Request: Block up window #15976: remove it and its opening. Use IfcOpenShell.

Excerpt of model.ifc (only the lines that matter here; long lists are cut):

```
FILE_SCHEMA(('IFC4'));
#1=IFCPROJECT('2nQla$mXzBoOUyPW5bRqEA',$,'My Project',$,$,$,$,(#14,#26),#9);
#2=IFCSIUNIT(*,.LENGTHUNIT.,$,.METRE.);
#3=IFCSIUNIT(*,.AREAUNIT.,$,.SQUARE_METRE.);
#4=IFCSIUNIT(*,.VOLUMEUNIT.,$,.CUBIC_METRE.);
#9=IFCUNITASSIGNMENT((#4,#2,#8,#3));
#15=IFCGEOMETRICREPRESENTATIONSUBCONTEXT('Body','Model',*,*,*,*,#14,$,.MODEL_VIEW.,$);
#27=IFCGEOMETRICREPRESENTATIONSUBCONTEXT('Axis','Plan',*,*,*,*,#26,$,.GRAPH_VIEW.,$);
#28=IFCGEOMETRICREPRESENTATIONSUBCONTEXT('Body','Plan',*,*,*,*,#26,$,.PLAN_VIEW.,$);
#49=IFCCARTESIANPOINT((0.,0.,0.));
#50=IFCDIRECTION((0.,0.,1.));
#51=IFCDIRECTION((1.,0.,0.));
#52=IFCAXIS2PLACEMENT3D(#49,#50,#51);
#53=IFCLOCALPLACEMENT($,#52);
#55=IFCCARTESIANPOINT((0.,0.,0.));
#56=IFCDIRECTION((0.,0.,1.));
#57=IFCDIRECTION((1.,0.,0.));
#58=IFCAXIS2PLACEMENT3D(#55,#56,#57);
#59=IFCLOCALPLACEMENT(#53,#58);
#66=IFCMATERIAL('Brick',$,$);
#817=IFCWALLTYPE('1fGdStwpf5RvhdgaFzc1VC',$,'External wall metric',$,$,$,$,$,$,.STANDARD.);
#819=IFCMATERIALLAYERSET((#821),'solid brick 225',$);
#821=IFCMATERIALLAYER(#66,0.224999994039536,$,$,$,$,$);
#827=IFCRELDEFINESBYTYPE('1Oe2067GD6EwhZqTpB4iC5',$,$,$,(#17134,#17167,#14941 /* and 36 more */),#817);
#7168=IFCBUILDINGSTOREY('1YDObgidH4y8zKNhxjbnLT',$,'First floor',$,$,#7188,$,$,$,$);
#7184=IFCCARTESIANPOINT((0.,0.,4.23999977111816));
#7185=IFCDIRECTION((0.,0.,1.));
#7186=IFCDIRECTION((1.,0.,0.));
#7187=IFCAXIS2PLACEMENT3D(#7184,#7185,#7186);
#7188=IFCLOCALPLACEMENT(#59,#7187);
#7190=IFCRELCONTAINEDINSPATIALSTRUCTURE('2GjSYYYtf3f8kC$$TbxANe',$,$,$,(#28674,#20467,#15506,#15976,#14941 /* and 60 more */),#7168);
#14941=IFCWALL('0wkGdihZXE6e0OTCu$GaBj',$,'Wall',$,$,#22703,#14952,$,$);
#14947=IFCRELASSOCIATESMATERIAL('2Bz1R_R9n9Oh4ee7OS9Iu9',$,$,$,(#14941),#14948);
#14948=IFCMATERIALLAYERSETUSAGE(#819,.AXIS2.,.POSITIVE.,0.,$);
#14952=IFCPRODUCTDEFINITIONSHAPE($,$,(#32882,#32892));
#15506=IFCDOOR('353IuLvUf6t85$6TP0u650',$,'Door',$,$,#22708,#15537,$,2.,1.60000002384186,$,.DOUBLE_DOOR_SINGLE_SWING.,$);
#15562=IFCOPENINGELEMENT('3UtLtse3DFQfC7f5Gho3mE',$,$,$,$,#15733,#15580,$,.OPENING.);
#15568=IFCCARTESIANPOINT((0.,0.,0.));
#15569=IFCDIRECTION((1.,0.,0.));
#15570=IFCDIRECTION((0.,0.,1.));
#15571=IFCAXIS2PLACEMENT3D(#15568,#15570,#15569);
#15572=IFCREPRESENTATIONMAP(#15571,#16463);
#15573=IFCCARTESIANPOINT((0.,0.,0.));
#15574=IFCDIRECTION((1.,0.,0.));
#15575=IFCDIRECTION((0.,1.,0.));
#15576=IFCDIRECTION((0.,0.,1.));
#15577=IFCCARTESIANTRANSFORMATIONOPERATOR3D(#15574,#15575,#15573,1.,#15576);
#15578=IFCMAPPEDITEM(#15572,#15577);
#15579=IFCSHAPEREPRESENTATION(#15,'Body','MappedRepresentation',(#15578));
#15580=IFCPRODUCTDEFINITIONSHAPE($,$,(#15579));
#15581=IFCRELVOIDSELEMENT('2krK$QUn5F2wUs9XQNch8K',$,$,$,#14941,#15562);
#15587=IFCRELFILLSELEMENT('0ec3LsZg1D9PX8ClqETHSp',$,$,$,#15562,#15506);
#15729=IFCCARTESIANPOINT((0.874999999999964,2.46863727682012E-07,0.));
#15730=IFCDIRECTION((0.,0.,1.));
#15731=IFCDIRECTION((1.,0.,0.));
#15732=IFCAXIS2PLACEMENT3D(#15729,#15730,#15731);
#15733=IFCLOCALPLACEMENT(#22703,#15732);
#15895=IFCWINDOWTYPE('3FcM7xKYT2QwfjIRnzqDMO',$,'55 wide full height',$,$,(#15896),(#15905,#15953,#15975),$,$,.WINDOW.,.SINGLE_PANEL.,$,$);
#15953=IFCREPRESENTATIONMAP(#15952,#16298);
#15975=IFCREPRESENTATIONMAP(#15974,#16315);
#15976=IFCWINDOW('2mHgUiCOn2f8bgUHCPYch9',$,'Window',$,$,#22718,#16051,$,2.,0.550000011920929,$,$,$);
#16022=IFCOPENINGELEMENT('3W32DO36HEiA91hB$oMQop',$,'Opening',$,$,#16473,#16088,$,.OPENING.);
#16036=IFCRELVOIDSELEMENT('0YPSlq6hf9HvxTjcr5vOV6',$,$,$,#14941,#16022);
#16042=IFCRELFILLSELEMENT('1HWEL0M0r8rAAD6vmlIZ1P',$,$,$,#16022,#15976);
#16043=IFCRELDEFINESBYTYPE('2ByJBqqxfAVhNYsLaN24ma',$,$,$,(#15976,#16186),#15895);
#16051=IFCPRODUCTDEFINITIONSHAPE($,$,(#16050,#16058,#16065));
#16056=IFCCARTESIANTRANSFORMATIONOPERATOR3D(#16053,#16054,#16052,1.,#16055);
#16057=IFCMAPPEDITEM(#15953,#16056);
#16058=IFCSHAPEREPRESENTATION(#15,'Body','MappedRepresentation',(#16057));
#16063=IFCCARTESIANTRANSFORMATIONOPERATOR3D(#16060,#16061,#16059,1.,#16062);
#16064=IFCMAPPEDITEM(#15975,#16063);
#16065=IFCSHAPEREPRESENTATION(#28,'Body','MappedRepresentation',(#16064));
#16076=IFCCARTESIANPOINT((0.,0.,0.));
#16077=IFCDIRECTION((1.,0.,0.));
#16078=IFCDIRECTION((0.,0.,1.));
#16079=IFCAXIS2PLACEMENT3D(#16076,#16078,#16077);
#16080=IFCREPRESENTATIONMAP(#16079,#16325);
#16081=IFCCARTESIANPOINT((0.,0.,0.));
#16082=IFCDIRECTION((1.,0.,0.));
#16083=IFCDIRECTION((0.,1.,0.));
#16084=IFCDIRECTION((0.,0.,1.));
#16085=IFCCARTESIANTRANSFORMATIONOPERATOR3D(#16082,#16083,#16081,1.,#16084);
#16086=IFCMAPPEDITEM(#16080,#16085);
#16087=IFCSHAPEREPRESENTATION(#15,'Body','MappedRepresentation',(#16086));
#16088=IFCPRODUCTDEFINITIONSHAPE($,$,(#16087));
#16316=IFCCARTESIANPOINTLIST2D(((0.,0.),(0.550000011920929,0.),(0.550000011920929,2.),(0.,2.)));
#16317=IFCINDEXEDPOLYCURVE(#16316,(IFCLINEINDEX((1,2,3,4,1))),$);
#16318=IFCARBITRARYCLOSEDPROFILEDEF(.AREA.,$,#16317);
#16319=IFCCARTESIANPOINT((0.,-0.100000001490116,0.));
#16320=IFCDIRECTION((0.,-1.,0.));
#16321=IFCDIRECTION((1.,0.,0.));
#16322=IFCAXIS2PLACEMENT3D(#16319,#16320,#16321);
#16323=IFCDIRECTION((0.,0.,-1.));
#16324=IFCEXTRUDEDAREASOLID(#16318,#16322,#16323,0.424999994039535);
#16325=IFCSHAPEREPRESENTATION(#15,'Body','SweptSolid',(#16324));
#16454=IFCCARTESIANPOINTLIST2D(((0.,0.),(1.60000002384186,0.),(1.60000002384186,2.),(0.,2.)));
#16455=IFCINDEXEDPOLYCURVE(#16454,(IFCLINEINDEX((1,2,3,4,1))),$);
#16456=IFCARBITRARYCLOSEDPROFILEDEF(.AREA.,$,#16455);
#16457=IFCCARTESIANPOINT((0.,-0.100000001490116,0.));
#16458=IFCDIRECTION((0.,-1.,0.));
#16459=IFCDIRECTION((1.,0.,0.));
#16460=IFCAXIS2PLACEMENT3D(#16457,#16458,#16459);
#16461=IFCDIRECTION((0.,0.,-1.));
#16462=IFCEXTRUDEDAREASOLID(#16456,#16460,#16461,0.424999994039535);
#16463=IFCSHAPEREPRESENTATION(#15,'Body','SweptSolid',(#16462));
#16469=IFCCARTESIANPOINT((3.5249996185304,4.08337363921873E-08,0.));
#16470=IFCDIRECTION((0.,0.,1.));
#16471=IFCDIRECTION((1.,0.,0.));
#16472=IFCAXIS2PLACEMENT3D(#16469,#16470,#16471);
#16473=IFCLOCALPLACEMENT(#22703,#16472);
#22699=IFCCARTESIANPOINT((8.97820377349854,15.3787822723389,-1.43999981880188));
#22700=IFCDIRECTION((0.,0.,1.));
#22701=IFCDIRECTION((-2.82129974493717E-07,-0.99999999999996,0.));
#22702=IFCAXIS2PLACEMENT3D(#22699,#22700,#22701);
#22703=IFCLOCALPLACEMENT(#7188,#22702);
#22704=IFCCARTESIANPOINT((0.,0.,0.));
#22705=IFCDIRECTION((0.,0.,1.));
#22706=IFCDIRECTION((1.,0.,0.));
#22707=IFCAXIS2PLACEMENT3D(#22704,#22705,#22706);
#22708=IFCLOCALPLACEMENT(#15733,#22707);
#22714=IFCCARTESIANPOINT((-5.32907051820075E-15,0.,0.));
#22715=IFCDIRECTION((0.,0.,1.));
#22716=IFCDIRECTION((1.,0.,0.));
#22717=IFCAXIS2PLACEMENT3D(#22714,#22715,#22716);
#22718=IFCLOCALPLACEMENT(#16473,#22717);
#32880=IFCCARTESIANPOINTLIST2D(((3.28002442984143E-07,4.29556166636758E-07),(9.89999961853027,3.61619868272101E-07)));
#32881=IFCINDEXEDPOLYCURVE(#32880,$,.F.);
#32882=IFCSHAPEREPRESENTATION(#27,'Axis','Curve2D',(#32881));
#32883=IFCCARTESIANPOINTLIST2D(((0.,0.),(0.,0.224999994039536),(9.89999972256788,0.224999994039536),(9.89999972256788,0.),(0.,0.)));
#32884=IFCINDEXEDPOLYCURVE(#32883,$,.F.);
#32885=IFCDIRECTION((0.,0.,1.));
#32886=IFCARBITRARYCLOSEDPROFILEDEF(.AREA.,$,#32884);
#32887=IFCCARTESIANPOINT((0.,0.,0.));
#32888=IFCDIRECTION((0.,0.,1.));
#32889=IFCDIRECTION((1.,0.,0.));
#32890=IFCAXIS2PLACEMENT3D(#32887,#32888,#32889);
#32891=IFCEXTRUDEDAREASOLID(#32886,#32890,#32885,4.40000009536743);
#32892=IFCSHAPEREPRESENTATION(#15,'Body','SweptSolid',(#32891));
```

```python
import ifcopenshell
import ifcopenshell.api.feature
import ifcopenshell.api.root
import ifcopenshell.geom
import ifcopenshell.util.shape

model = ifcopenshell.open("model.ifc")
settings = ifcopenshell.geom.settings()


def volume(element):
    """Net volume in cubic metres, openings subtracted."""
    shape = ifcopenshell.geom.create_shape(settings, element)
    return ifcopenshell.util.shape.get_volume(shape.geometry)


window = model.by_guid("2mHgUiCOn2f8bgUHCPYch9")
opening = window.FillsVoids[0].RelatingOpeningElement
wall = opening.VoidsElements[0].RelatingBuildingElement
before = volume(wall)

ifcopenshell.api.root.remove_product(model, product=window)
ifcopenshell.api.feature.remove_feature(model, feature=opening)

after = volume(wall)

print(f"wall volume {before:.3f} -> {after:.3f} m3")

model.write("model_rev.ifc")
```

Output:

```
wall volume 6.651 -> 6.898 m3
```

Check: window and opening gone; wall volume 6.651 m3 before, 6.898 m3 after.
